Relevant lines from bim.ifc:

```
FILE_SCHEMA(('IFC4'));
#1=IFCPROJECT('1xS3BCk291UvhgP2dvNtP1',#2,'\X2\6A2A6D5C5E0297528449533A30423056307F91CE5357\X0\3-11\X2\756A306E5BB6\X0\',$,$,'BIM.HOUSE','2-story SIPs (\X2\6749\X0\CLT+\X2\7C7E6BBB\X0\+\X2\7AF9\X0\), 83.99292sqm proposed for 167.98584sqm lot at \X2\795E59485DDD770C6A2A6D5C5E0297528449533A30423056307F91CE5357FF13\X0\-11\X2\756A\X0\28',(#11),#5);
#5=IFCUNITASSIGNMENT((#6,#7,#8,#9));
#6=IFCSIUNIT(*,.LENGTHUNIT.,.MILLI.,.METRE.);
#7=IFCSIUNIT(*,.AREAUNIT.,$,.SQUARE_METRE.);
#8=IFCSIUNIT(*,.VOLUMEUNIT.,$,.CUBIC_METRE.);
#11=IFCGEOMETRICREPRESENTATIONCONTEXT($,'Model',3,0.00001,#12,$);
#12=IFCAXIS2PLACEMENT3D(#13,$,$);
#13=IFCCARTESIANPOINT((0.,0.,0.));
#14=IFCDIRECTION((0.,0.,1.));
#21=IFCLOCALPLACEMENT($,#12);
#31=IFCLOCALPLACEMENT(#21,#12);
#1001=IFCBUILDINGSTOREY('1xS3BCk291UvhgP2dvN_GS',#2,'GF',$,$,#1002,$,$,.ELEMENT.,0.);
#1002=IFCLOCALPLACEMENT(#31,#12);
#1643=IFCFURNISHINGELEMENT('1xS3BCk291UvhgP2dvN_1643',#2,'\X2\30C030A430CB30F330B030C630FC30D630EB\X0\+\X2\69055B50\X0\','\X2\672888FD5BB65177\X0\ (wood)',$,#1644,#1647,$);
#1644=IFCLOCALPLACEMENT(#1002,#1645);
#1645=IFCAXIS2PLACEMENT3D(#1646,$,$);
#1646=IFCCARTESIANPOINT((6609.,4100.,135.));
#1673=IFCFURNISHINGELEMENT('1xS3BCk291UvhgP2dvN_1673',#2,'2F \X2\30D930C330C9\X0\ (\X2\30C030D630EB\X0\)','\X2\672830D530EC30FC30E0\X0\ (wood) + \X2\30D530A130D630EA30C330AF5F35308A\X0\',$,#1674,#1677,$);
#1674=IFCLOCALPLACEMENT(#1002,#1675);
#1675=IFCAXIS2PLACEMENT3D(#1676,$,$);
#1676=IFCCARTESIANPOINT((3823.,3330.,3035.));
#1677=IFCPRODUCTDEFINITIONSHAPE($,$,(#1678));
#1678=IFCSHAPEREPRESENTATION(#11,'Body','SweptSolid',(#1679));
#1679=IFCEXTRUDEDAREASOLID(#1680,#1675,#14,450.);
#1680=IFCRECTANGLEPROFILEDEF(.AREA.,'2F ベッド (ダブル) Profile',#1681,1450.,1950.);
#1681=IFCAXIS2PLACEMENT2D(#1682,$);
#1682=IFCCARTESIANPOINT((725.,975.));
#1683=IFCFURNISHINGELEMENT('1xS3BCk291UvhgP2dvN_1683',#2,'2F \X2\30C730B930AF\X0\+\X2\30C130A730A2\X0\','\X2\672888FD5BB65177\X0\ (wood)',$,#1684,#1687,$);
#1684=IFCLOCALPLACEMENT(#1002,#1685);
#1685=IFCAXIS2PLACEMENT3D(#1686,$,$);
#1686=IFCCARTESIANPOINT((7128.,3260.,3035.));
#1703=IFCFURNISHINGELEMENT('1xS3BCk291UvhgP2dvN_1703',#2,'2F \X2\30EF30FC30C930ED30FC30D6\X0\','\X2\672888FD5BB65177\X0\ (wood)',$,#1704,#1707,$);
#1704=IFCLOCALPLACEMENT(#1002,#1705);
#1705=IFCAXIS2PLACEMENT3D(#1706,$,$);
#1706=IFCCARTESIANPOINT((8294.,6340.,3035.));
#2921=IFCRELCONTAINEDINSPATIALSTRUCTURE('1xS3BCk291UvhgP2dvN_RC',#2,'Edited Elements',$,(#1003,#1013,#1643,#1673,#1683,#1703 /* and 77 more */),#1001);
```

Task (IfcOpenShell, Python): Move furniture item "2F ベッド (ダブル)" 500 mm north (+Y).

```python
import ifcopenshell
import ifcopenshell.api.geometry
import ifcopenshell.util.placement
import ifcopenshell.util.unit

model = ifcopenshell.open("bim.ifc")
unit_scale = ifcopenshell.util.unit.calculate_unit_scale(model)

item = model.by_id(1673)
matrix = ifcopenshell.util.placement.get_local_placement(item.ObjectPlacement)
matrix[1, 3] += 0.5 / unit_scale
ifcopenshell.api.geometry.edit_object_placement(model, product=item, matrix=matrix, is_si=False)

print(ifcopenshell.util.placement.get_local_placement(item.ObjectPlacement).round(3) + 0.0)

model.write("bim_rev.ifc")
```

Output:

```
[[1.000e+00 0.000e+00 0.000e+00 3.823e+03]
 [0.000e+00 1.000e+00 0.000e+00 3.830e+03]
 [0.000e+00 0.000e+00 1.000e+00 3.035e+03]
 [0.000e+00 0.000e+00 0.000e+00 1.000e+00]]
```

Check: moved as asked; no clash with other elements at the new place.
